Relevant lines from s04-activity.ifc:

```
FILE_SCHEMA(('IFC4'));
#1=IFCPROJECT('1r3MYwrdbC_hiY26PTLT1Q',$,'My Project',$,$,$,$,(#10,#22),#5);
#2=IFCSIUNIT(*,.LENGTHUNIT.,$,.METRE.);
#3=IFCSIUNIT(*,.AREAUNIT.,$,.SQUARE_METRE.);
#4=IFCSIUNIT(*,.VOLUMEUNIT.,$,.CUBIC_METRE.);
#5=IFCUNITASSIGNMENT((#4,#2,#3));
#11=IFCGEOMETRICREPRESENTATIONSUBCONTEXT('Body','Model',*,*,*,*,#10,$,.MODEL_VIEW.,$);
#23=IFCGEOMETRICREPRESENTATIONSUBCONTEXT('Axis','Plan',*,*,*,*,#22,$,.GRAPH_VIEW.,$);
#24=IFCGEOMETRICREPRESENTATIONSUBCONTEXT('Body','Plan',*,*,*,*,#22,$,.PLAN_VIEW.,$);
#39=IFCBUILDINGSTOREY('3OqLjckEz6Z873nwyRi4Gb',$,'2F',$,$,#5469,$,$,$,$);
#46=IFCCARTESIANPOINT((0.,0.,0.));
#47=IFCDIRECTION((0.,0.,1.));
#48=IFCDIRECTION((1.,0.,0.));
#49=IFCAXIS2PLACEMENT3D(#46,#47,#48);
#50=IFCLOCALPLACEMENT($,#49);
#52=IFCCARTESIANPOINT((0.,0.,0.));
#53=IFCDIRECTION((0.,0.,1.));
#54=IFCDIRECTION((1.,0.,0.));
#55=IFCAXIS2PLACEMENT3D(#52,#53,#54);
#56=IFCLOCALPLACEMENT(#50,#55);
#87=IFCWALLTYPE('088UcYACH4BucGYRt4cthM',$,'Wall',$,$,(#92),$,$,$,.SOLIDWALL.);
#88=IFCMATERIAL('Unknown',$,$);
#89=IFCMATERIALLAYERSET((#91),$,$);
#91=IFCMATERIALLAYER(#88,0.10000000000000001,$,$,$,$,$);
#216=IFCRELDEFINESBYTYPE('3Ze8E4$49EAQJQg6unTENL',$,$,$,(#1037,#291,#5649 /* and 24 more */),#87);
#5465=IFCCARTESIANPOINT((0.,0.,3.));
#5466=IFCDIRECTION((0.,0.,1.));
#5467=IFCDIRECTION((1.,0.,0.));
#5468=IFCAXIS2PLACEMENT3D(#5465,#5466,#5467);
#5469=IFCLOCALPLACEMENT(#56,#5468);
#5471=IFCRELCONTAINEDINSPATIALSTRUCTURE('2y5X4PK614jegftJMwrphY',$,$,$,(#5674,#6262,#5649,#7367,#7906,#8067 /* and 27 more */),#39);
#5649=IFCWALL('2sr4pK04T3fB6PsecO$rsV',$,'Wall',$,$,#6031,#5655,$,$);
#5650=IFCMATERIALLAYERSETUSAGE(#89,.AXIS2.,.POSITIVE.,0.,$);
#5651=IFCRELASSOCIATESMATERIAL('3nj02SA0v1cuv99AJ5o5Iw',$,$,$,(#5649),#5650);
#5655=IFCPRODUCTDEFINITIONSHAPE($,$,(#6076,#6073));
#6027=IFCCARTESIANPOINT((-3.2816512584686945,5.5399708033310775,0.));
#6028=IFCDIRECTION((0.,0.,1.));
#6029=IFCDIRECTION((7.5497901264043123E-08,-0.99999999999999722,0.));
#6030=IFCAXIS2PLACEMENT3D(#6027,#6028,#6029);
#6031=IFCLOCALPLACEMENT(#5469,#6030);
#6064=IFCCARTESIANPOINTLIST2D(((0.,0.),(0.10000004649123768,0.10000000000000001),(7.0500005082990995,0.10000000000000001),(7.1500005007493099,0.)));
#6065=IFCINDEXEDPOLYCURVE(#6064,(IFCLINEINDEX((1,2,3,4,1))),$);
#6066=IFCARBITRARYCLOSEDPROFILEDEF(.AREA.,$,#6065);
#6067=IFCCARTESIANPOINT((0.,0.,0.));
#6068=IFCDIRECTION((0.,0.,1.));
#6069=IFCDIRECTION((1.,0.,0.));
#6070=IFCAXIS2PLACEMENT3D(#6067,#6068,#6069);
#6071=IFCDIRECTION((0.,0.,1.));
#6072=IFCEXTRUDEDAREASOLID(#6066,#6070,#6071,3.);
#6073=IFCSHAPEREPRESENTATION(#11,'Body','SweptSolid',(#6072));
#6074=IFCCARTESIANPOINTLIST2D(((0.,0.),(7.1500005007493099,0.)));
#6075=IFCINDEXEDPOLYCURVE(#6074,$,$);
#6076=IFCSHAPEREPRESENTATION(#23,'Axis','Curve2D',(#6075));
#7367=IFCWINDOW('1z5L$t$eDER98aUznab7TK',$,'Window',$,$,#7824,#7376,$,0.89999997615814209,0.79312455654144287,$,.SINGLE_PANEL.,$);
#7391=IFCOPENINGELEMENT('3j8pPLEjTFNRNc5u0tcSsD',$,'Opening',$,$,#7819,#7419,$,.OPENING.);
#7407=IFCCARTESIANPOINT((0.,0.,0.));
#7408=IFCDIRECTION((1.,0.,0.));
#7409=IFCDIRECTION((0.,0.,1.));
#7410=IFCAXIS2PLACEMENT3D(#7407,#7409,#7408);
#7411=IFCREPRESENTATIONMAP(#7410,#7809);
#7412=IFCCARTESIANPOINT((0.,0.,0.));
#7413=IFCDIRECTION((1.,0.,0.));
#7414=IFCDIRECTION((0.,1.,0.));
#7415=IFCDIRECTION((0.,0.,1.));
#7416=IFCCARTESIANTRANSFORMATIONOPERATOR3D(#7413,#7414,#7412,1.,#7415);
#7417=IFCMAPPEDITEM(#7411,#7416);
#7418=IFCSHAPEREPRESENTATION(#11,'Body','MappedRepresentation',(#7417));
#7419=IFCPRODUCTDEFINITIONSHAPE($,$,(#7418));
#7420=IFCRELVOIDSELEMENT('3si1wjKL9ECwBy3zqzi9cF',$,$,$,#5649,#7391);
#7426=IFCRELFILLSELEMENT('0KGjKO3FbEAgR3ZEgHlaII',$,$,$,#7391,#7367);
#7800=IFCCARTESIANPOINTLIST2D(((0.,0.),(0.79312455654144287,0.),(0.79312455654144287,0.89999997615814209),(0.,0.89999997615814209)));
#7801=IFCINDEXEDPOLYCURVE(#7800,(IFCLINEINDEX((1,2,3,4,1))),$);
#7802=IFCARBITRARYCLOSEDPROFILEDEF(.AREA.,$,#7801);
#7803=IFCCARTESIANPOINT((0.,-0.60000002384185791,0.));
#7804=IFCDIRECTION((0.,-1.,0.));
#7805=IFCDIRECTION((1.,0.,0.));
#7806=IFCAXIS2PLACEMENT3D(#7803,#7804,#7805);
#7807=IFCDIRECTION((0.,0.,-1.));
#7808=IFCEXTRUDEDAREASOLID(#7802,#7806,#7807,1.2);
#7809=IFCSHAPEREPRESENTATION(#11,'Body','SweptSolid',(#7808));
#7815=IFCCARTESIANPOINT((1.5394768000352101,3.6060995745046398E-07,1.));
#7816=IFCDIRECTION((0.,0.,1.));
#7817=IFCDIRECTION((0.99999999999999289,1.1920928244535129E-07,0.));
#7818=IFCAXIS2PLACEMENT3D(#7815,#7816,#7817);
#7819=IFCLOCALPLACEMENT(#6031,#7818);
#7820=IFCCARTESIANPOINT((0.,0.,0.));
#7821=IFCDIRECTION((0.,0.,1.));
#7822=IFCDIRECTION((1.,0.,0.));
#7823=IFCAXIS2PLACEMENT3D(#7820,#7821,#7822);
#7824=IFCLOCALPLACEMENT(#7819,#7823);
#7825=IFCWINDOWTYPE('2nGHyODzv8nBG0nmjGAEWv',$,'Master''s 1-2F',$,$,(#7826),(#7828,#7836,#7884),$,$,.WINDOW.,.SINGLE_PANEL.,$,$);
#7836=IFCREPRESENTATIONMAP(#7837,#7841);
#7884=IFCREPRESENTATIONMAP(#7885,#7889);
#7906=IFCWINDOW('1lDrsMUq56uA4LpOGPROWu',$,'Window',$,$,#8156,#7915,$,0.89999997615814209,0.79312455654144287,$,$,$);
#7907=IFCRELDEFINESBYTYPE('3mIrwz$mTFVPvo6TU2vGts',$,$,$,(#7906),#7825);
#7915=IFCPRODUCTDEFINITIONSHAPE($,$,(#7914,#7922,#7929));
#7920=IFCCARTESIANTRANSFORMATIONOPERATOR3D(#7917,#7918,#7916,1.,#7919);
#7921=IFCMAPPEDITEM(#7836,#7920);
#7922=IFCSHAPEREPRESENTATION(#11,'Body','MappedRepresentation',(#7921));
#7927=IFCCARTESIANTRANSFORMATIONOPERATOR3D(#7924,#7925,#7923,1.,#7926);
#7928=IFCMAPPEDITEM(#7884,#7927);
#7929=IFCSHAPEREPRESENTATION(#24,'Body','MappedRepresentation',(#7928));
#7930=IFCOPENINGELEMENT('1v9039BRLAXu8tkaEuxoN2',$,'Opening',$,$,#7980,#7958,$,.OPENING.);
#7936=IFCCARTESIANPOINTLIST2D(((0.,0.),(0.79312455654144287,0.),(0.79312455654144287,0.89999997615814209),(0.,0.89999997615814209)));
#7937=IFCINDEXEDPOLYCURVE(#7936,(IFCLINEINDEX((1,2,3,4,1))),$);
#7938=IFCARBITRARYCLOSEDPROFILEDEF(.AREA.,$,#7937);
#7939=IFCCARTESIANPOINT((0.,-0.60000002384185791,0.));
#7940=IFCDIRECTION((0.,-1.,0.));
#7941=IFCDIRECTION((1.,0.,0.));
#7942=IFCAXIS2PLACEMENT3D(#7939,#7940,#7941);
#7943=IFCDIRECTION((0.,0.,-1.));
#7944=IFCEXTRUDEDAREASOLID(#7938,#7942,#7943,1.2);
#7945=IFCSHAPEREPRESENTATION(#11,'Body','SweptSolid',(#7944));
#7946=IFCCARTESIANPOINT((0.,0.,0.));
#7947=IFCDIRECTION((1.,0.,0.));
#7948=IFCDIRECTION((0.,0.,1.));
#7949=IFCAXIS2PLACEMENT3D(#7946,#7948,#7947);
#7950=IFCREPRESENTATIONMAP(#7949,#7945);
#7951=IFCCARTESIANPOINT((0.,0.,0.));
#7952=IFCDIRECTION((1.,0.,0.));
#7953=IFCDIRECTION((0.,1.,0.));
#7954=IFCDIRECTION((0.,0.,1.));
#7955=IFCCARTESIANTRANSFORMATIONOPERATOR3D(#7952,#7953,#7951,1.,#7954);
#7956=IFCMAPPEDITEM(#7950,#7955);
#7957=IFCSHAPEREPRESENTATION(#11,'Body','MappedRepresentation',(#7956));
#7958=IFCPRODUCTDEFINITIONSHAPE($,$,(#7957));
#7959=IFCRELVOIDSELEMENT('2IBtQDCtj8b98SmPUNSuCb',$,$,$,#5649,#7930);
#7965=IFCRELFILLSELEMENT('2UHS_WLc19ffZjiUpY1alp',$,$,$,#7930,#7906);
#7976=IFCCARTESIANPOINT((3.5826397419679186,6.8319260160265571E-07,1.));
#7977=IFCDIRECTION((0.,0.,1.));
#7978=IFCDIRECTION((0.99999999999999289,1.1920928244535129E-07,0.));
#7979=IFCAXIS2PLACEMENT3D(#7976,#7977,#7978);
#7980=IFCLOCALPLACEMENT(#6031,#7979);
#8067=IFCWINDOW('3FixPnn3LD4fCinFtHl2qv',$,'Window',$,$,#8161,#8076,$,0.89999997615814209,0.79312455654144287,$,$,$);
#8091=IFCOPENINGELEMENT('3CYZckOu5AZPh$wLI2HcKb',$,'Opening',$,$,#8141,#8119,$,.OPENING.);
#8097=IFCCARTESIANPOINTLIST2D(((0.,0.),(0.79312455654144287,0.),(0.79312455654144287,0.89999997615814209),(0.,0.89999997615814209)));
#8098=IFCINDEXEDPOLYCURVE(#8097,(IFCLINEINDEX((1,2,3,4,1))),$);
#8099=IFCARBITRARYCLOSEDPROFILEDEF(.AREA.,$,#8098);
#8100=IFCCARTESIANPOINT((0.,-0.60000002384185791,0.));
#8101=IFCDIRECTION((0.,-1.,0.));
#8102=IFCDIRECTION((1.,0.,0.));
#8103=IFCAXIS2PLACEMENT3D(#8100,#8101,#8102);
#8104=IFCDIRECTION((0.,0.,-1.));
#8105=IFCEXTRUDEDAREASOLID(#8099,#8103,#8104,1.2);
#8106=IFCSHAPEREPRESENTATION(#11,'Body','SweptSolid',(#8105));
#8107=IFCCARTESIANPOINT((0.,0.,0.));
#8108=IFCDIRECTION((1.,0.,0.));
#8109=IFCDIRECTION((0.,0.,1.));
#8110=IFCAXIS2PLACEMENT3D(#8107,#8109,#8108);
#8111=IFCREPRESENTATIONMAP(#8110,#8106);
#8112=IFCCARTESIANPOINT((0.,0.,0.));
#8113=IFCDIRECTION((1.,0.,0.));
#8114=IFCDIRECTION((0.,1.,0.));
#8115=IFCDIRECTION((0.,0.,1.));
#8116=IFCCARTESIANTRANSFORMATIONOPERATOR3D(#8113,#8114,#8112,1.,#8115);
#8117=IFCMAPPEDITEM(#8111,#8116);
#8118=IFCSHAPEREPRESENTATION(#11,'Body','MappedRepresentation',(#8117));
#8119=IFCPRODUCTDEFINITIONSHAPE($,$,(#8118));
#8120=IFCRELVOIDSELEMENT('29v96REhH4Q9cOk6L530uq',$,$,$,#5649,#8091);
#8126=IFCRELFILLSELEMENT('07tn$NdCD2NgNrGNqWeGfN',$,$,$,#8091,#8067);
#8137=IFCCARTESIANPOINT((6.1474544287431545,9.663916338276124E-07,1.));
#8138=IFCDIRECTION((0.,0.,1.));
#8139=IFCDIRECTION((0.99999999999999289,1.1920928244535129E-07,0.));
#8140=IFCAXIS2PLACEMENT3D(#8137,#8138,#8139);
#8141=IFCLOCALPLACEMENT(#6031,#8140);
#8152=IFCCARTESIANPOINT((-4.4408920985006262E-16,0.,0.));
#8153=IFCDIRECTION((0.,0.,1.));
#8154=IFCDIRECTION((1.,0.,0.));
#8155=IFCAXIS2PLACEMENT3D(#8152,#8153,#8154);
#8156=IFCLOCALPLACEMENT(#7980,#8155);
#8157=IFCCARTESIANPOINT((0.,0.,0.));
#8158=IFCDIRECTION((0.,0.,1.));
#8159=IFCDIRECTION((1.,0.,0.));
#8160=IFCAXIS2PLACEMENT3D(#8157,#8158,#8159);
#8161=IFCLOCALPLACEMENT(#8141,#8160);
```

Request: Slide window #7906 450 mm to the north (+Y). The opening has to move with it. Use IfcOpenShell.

```python
import ifcopenshell
import ifcopenshell.api.geometry
import ifcopenshell.util.placement

model = ifcopenshell.open("s04-activity.ifc")

window = model.by_guid("1lDrsMUq56uA4LpOGPROWu")
opening = window.FillsVoids[0].RelatingOpeningElement
wall = opening.VoidsElements[0].RelatingBuildingElement

wall_matrix = ifcopenshell.util.placement.get_local_placement(wall.ObjectPlacement)
shift = wall_matrix[:3, 0] * -0.45
before = ifcopenshell.util.placement.get_local_placement(window.ObjectPlacement)[:3, 3].copy()

# The window is placed relative to its opening, so it follows when the opening moves.
matrix = ifcopenshell.util.placement.get_local_placement(opening.ObjectPlacement)
matrix[:3, 3] += shift
ifcopenshell.api.geometry.edit_object_placement(
    model, product=opening, matrix=matrix, is_si=False, should_transform_children=True
)

after = ifcopenshell.util.placement.get_local_placement(window.ObjectPlacement)[:3, 3]
print("window moved by", (after - before).round(3) + 0.0)

model.write("s04-activity_updated.ifc")
```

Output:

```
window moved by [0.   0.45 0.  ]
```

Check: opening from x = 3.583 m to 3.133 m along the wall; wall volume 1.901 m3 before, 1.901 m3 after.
